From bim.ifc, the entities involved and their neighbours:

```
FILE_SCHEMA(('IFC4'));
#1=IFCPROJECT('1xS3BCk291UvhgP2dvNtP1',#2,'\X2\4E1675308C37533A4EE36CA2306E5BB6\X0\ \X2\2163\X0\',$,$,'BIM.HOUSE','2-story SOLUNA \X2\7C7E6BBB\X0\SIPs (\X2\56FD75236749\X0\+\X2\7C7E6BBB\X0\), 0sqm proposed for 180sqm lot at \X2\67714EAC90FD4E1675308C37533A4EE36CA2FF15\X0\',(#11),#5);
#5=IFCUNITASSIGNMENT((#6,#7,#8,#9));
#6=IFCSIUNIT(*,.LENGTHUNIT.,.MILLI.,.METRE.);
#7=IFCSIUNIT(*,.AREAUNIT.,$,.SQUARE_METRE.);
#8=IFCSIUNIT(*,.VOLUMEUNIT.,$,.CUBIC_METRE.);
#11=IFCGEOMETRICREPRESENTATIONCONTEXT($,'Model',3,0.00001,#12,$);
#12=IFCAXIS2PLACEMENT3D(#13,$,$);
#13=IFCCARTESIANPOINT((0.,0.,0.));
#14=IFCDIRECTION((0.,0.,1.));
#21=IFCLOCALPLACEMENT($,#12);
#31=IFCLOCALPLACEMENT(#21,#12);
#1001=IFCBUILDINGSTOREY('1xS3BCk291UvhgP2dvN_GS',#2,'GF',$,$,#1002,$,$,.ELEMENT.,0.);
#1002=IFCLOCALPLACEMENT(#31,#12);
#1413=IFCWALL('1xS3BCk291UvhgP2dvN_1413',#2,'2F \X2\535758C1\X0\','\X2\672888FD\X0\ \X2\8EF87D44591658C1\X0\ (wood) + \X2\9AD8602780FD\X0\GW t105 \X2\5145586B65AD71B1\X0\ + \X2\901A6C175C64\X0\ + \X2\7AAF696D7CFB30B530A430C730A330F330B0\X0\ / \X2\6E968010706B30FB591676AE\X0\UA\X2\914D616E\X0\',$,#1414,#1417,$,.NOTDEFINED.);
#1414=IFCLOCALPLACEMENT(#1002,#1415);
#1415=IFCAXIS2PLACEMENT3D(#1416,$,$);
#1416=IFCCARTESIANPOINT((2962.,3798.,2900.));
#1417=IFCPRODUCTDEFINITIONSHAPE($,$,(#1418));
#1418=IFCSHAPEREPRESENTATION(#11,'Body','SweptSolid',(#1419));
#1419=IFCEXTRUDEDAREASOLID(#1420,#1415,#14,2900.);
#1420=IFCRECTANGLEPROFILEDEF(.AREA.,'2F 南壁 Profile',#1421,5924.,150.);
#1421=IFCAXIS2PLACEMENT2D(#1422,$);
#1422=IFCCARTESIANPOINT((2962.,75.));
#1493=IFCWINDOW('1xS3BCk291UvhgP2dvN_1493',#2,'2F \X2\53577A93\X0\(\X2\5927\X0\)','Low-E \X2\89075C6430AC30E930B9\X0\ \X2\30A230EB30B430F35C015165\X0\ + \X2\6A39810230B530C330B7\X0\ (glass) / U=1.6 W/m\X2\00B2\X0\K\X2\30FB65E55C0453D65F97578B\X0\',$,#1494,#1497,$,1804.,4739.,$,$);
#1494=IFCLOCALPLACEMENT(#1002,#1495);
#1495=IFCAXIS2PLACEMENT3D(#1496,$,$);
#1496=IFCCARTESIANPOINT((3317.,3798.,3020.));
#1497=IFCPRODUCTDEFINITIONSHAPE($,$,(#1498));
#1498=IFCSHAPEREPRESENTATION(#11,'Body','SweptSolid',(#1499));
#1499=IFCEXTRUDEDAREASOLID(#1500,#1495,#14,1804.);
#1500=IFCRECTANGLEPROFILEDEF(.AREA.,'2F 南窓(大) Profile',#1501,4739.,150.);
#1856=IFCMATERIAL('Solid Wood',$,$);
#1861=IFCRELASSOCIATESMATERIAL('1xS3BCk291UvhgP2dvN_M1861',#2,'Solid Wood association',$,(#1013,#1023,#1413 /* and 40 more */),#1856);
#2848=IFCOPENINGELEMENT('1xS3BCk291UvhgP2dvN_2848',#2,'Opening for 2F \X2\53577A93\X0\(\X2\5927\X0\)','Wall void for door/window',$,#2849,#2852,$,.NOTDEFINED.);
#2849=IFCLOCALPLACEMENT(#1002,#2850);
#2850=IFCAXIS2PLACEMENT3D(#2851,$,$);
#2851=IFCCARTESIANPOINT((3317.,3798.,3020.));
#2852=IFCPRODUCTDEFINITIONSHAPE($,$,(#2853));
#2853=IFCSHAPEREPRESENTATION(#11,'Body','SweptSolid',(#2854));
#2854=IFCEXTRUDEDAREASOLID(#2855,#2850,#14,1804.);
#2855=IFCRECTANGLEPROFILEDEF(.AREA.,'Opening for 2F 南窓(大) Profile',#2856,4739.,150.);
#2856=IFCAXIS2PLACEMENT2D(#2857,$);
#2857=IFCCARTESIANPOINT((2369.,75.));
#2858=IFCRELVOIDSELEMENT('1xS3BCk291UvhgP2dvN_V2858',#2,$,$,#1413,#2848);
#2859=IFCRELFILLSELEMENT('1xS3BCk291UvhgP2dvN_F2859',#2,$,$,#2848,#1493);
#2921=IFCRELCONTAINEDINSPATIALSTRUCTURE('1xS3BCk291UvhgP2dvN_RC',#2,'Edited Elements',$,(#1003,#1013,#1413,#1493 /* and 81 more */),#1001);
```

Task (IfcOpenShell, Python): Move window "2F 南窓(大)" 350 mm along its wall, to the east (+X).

```python
import ifcopenshell
import ifcopenshell.api.geometry
import ifcopenshell.util.placement
import ifcopenshell.util.unit

model = ifcopenshell.open("bim.ifc")
unit_scale = ifcopenshell.util.unit.calculate_unit_scale(model)

window = model.by_id(1493)
opening = window.FillsVoids[0].RelatingOpeningElement
wall = opening.VoidsElements[0].RelatingBuildingElement

wall_matrix = ifcopenshell.util.placement.get_local_placement(wall.ObjectPlacement)
shift = wall_matrix[:3, 0] * 0.35 / unit_scale
before = ifcopenshell.util.placement.get_local_placement(window.ObjectPlacement)[:3, 3].copy()

# The window is not placed relative to its opening, so move both.
for product in (opening, window):
    matrix = ifcopenshell.util.placement.get_local_placement(product.ObjectPlacement)
    matrix[:3, 3] += shift
    ifcopenshell.api.geometry.edit_object_placement(model, product=product, matrix=matrix, is_si=False)

after = ifcopenshell.util.placement.get_local_placement(window.ObjectPlacement)[:3, 3]
print("window moved by", (after - before).round(3) + 0.0)

model.write("bim_updated.ifc")
```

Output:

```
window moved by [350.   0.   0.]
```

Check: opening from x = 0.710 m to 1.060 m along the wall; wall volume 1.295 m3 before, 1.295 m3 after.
